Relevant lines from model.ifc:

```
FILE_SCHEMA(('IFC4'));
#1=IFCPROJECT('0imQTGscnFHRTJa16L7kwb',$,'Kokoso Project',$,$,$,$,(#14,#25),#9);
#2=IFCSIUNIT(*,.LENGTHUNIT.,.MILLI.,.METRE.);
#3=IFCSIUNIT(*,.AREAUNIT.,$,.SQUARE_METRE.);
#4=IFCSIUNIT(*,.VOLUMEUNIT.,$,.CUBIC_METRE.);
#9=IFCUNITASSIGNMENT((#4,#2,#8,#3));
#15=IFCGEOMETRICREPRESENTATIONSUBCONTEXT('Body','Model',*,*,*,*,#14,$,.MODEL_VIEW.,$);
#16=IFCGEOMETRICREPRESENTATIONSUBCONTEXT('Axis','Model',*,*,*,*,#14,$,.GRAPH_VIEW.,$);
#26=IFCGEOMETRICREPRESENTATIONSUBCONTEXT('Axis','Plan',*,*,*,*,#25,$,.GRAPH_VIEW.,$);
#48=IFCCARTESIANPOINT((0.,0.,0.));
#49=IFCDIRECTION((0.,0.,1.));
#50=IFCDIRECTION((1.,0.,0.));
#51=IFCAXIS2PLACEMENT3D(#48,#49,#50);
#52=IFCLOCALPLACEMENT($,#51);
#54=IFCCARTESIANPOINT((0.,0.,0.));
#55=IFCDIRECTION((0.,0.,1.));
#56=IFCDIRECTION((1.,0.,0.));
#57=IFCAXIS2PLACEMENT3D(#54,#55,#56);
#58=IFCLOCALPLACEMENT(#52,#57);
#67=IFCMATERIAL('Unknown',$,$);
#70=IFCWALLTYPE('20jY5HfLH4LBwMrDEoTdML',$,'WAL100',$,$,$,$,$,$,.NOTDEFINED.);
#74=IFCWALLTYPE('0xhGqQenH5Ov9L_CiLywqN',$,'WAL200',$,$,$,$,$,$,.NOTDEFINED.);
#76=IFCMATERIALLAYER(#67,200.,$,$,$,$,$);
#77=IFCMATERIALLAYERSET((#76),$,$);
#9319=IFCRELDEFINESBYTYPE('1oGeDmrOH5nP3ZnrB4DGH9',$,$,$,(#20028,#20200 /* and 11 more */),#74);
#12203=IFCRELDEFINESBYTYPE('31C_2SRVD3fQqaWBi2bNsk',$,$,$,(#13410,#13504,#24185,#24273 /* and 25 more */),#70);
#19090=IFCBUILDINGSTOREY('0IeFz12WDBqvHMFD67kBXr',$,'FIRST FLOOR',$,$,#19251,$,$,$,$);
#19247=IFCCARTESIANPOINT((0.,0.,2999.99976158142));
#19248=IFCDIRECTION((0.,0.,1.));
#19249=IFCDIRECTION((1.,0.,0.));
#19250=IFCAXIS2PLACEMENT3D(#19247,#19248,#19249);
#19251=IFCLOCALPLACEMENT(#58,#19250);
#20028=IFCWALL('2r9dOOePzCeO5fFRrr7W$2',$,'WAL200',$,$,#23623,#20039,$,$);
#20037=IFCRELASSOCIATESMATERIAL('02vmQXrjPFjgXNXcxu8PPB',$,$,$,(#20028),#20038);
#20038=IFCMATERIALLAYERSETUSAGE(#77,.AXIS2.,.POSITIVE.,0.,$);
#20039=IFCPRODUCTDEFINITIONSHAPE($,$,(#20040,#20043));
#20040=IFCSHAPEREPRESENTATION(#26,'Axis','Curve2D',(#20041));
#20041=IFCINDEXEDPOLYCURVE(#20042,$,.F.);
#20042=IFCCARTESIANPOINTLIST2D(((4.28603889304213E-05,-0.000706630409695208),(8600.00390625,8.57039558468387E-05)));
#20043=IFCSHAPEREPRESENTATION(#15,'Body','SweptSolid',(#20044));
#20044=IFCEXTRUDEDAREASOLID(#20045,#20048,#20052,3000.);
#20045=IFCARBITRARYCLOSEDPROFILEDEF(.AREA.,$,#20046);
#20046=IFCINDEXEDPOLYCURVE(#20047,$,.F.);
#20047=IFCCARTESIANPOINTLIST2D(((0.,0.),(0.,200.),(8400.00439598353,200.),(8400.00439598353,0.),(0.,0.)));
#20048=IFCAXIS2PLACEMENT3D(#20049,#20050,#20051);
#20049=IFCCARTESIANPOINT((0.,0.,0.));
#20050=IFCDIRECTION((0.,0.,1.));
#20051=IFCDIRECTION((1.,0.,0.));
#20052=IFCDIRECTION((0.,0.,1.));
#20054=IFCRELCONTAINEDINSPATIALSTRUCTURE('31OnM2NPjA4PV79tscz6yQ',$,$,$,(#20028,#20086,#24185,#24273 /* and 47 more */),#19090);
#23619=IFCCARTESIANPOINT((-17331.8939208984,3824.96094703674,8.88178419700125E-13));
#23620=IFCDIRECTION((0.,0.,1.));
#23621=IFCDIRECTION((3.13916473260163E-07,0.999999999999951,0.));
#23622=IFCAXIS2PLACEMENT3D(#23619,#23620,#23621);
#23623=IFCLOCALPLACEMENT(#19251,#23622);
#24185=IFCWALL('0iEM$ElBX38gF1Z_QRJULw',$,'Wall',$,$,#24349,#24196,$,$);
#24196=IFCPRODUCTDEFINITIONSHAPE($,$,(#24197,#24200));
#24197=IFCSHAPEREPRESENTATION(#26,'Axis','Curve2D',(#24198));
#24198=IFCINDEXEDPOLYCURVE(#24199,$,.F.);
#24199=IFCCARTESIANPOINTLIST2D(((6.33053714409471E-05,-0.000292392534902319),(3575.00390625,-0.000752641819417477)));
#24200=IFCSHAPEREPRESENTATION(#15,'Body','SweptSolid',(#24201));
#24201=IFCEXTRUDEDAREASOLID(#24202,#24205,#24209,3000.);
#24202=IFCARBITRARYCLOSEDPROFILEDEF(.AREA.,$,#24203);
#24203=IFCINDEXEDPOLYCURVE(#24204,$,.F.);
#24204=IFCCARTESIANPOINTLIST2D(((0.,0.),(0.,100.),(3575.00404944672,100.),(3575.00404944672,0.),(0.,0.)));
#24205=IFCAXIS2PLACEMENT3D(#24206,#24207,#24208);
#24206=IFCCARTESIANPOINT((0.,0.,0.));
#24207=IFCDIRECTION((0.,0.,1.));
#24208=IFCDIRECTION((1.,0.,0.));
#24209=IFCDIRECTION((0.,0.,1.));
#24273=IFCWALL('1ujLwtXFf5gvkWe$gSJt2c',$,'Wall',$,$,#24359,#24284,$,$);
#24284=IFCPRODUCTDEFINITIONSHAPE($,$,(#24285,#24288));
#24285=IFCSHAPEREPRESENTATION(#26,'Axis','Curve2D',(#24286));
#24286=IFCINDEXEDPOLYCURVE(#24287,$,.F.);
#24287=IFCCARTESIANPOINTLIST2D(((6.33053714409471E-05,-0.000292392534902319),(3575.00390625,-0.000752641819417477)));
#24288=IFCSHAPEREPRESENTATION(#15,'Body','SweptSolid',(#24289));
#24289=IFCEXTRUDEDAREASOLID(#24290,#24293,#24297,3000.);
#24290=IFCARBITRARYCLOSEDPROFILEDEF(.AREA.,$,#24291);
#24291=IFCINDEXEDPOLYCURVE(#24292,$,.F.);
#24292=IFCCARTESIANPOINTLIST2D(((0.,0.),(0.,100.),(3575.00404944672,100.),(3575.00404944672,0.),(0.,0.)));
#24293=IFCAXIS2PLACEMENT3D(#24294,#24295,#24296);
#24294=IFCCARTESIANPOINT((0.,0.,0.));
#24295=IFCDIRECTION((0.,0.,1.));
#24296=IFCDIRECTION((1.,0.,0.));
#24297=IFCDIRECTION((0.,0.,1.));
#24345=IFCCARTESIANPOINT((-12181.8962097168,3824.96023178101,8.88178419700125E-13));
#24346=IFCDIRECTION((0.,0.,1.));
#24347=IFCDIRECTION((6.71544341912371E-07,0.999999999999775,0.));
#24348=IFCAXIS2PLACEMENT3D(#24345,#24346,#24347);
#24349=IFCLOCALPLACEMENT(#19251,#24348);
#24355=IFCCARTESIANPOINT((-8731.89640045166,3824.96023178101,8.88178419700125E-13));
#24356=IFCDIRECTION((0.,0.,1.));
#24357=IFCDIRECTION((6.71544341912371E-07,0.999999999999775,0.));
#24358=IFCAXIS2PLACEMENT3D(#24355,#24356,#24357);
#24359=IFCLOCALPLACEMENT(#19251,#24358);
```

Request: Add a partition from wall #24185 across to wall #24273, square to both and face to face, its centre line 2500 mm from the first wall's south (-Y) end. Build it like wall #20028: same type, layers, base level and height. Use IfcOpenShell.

```python
import numpy as np
import ifcopenshell
import ifcopenshell.api.geometry
import ifcopenshell.api.material
import ifcopenshell.api.pset
import ifcopenshell.api.root
import ifcopenshell.api.spatial
import ifcopenshell.api.type
import ifcopenshell.geom
import ifcopenshell.util.element
import ifcopenshell.util.placement
import ifcopenshell.util.representation
import ifcopenshell.util.shape
import ifcopenshell.util.unit

model = ifcopenshell.open("model.ifc")
unit_scale = ifcopenshell.util.unit.calculate_unit_scale(model)
settings = ifcopenshell.geom.settings()
settings.set("use-world-coords", True)

start_wall = model.by_id(24185)
end_wall = model.by_id(24273)
like = model.by_id(20028)
matrix = ifcopenshell.util.placement.get_local_placement(start_wall.ObjectPlacement)
matrix[:3, 3] *= unit_scale


def extent(element):
    """Bounding box in the first wall's axes, in metres."""
    shape = ifcopenshell.geom.create_shape(settings, element)
    points = (ifcopenshell.util.shape.get_vertices(shape.geometry) - matrix[:3, 3]) @ matrix[:3, :3]
    return points.min(axis=0), points.max(axis=0)


y_start = extent(start_wall)[0][1]
y_end = extent(end_wall)[1][1]
like_min, like_max = extent(like)
length, height = float(abs(y_end - y_start)), float(like_max[2] - like_min[2])
layer_set = ifcopenshell.util.element.get_material(like, should_skip_usage=True)
thickness = sum(layer.LayerThickness for layer in layer_set.MaterialLayers) * unit_scale

wall = ifcopenshell.api.root.create_entity(model, ifc_class="IfcWall", name="New partition")
storey = ifcopenshell.util.element.get_container(like)
ifcopenshell.api.spatial.assign_container(model, products=[wall], relating_structure=storey)
ifcopenshell.api.type.assign_type(
    model, related_objects=[wall], relating_type=ifcopenshell.util.element.get_type(like), should_map_representations=False
)
rel = ifcopenshell.api.material.assign_material(
    model, products=[wall], type="IfcMaterialLayerSetUsage", material=layer_set
)
rel.RelatingMaterial.OffsetFromReferenceLine = -thickness / 2 / unit_scale
pset = ifcopenshell.api.pset.add_pset(model, product=wall, name="Pset_WallCommon")
ifcopenshell.api.pset.edit_pset(model, pset=pset, properties={"IsExternal": False, "LoadBearing": False})

# The axis runs down the middle of the wall.
axis = ifcopenshell.api.geometry.add_axis_representation(
    model, context=ifcopenshell.util.representation.get_context(model, "Model", "Axis"), axis=[(0.0, 0.0), (length, 0.0)]
)
body = ifcopenshell.api.geometry.add_wall_representation(
    model,
    context=ifcopenshell.util.representation.get_context(model, "Model", "Body", "MODEL_VIEW"),
    length=length,
    height=height,
    thickness=thickness,
    offset=-thickness / 2,
)
for representation in (axis, body):
    ifcopenshell.api.geometry.assign_representation(model, product=wall, representation=representation)

placement = matrix @ ifcopenshell.util.placement.rotation(-90, "Z")
placement[:, 3] = matrix @ np.array([extent(start_wall)[0][0] + 2.5, y_start, like_min[2], 1.0])
ifcopenshell.api.geometry.edit_object_placement(model, product=wall, matrix=placement)

print(f"partition {length:.3f} m long, {height:.3f} m high, {thickness:.3f} m thick")

model.write("model_updated.ifc")
```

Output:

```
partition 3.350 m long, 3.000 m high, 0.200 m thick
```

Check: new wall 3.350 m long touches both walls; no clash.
